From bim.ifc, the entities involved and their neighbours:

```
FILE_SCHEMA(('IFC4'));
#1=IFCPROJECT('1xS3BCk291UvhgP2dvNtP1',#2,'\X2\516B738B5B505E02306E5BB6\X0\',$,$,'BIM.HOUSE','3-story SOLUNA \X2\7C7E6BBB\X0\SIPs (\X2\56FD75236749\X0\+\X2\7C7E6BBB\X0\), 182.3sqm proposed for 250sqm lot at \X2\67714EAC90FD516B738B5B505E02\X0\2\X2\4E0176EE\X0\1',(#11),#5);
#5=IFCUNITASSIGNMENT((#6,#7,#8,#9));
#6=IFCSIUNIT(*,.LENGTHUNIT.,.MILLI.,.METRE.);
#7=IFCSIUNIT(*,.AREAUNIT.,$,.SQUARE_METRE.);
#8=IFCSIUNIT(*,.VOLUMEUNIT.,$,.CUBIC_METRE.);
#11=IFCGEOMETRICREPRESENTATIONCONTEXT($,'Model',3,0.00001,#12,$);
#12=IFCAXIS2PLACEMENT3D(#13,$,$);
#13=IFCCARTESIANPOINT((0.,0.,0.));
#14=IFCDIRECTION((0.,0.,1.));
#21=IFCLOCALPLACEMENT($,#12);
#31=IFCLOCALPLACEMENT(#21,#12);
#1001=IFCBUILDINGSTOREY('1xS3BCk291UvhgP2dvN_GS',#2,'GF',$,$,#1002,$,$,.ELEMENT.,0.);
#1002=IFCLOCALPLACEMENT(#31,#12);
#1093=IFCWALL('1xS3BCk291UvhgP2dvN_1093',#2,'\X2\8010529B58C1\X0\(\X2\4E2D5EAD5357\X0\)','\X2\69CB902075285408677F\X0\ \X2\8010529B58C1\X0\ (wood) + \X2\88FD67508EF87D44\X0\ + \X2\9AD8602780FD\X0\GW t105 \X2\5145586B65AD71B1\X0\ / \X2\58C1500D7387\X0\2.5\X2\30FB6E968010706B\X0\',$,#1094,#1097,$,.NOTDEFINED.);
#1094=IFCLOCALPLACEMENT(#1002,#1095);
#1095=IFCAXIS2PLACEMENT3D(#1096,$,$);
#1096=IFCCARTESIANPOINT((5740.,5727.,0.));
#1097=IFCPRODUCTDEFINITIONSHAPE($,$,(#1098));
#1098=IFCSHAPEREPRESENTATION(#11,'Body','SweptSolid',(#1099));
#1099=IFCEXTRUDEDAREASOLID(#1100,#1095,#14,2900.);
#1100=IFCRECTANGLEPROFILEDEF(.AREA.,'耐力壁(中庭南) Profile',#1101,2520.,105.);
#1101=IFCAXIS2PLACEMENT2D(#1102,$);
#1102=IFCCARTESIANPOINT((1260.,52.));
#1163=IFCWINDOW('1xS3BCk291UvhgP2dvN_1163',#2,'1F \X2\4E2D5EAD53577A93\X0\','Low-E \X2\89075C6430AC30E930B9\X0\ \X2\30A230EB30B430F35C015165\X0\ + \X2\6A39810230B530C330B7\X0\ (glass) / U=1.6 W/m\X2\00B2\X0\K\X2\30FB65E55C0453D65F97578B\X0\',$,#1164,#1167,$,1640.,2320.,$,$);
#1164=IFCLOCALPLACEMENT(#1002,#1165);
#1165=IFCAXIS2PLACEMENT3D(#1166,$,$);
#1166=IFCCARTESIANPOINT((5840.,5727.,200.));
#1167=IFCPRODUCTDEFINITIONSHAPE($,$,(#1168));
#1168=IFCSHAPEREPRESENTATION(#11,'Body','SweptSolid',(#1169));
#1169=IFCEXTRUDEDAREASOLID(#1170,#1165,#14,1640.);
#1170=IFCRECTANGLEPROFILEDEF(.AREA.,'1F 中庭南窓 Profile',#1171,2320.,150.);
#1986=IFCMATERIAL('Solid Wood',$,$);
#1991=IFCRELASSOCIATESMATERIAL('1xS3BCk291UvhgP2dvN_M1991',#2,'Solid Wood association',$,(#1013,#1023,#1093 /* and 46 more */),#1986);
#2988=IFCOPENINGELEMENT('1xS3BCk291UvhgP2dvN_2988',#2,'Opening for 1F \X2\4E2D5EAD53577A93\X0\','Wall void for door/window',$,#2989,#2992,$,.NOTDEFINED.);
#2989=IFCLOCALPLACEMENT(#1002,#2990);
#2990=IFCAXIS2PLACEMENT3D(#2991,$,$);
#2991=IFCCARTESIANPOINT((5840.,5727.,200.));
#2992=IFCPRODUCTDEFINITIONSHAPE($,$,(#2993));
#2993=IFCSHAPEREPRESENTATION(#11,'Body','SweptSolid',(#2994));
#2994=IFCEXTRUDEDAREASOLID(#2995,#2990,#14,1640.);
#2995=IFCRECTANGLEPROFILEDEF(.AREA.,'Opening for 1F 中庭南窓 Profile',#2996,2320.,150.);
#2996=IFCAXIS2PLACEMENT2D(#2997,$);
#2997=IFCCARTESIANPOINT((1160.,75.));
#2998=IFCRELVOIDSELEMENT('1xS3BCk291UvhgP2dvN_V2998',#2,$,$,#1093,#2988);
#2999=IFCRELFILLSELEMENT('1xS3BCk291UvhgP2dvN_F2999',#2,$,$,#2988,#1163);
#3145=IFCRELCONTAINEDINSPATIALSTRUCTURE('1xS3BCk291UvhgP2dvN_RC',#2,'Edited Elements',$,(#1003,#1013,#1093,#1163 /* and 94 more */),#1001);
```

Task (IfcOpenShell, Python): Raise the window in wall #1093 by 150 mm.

```python
import numpy as np
import ifcopenshell
import ifcopenshell.api.geometry
import ifcopenshell.util.placement
import ifcopenshell.util.unit

model = ifcopenshell.open("bim.ifc")
unit_scale = ifcopenshell.util.unit.calculate_unit_scale(model)

window = model.by_guid("1xS3BCk291UvhgP2dvN_1163")
opening = window.FillsVoids[0].RelatingOpeningElement
dz = 150.0

shift = np.array([0.0, 0.0, dz])
# The window is not placed relative to its opening, so move both.
for product in (opening, window):
    matrix = ifcopenshell.util.placement.get_local_placement(product.ObjectPlacement)
    matrix[:3, 3] += shift
    ifcopenshell.api.geometry.edit_object_placement(model, product=product, matrix=matrix, is_si=False)

print(f"moved by {dz * unit_scale:+.3f} m")

model.write("bim_v2.ifc")
```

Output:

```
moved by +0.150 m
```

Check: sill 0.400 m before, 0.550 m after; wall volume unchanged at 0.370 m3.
